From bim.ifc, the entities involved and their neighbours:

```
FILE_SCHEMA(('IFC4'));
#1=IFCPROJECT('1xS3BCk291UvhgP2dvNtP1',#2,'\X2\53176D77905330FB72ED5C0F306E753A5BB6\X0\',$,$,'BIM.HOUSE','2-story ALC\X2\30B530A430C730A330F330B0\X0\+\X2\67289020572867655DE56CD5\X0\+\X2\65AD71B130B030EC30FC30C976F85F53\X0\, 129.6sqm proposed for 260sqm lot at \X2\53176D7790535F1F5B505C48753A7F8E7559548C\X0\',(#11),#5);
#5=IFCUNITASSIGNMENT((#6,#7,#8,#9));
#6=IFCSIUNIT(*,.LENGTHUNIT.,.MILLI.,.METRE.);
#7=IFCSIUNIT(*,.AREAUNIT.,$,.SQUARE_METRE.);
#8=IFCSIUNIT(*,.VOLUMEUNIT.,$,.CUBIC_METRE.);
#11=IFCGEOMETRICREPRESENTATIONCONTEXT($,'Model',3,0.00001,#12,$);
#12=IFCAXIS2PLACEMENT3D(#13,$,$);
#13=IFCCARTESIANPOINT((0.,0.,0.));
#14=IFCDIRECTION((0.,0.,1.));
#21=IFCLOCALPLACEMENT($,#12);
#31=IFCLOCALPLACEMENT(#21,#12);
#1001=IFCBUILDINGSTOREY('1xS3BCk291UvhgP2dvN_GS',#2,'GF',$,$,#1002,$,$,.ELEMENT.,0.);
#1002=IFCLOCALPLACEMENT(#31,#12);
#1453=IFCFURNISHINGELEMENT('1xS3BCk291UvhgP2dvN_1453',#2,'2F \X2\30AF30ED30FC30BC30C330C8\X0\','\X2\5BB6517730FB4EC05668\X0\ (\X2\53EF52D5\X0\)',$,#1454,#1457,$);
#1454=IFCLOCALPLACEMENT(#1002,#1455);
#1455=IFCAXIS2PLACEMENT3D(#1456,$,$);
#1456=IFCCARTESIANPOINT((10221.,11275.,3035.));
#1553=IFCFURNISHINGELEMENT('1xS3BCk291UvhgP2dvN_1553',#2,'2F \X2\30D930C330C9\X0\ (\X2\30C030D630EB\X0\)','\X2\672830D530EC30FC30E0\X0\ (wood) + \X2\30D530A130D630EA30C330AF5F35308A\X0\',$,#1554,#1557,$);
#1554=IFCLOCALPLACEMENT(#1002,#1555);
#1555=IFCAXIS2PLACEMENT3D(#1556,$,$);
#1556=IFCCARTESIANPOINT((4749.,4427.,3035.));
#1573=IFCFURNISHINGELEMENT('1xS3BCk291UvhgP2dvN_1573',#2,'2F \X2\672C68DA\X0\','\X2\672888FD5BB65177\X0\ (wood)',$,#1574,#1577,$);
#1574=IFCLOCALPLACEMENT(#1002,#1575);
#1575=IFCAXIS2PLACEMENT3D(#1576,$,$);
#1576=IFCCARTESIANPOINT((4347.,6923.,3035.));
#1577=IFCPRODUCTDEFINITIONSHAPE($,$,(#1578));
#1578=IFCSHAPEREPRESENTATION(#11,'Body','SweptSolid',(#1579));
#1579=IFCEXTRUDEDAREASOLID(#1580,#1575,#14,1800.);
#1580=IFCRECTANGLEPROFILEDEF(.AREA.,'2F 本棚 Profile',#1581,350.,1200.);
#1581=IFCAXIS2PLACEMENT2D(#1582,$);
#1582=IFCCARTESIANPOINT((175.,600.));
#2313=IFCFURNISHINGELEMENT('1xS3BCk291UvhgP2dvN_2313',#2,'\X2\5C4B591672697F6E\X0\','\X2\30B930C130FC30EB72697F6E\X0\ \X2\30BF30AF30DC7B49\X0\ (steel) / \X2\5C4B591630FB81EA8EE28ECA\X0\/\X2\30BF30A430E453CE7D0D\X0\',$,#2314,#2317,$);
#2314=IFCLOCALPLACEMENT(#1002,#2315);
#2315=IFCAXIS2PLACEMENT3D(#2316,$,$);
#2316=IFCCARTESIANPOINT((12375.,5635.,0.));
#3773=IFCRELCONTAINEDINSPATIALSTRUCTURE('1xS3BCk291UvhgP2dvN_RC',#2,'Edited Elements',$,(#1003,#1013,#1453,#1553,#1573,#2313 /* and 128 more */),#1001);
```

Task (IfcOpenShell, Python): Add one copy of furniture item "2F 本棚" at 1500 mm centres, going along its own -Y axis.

```python
import ifcopenshell
import ifcopenshell.api.geometry
import ifcopenshell.api.root
import ifcopenshell.util.element
import ifcopenshell.util.placement
import ifcopenshell.util.unit

model = ifcopenshell.open("bim.ifc")
unit_scale = ifcopenshell.util.unit.calculate_unit_scale(model)


def reuse_history(source, copy):
    """copy_class also copies each property set's owner history, people and application; keep the originals."""
    for rel in copy.IsDefinedBy:
        if rel.is_a("IfcRelDefinesByProperties") and (history := rel.RelatingPropertyDefinition.OwnerHistory):
            rel.RelatingPropertyDefinition.OwnerHistory = source.OwnerHistory
            ifcopenshell.util.element.remove_deep2(model, history)


source = model.by_guid("1xS3BCk291UvhgP2dvN_1573")
base = ifcopenshell.util.placement.get_local_placement(source.ObjectPlacement)
step = -base[:3, 1] * 1.5 / unit_scale

for i in range(1, 2):
    copy = ifcopenshell.api.root.copy_class(model, product=source)
    copy.Representation = ifcopenshell.util.element.copy_deep(
        model, source.Representation, exclude=["IfcGeometricRepresentationContext", "IfcRepresentationMap"]
    )
    reuse_history(source, copy)
    matrix = base.copy()
    matrix[:3, 3] += i * step
    print("added at", matrix[:3, 3].round(3) + 0.0)
    ifcopenshell.api.geometry.edit_object_placement(model, product=copy, matrix=matrix, is_si=False)

model.write("bim_updated.ifc")
```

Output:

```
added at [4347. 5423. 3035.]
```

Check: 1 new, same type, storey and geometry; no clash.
